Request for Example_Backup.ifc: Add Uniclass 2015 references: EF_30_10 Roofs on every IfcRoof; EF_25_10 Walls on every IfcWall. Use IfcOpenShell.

First a look at what the model holds.

```python
import ifcopenshell

model = ifcopenshell.open("Example_Backup.ifc")
print(model.schema)
print("classifications:", [c.Name for c in model.by_type("IfcClassification")])
for ifc_class in ("IfcDoor", "IfcRoof", "IfcStair", "IfcWall", "IfcWindow"):
    print(ifc_class, len(model.by_type(ifc_class)))
```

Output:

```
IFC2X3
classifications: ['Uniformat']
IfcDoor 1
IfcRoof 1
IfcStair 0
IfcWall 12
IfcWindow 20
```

```python
import ifcopenshell
import ifcopenshell.api.classification

model = ifcopenshell.open("Example_Backup.ifc")

# IFC2X3 requires Source and Edition and has no link from the project to the system.
system = model.create_entity("IfcClassification", Source="NBS", Edition="2015", Name="Uniclass 2015")

codes = {
    "IfcRoof": ("EF_30_10", "Roofs"),
    "IfcWall": ("EF_25_10", "Walls"),
}
for ifc_class, (code, name) in codes.items():
    products = model.by_type(ifc_class)
    ifcopenshell.api.classification.add_reference(
        model, products=products, classification=system, identification=code, name=name
    )
    print(code, len(products))

model.write("Example_Backup-out.ifc")
```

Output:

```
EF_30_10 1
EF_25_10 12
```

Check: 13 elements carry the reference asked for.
